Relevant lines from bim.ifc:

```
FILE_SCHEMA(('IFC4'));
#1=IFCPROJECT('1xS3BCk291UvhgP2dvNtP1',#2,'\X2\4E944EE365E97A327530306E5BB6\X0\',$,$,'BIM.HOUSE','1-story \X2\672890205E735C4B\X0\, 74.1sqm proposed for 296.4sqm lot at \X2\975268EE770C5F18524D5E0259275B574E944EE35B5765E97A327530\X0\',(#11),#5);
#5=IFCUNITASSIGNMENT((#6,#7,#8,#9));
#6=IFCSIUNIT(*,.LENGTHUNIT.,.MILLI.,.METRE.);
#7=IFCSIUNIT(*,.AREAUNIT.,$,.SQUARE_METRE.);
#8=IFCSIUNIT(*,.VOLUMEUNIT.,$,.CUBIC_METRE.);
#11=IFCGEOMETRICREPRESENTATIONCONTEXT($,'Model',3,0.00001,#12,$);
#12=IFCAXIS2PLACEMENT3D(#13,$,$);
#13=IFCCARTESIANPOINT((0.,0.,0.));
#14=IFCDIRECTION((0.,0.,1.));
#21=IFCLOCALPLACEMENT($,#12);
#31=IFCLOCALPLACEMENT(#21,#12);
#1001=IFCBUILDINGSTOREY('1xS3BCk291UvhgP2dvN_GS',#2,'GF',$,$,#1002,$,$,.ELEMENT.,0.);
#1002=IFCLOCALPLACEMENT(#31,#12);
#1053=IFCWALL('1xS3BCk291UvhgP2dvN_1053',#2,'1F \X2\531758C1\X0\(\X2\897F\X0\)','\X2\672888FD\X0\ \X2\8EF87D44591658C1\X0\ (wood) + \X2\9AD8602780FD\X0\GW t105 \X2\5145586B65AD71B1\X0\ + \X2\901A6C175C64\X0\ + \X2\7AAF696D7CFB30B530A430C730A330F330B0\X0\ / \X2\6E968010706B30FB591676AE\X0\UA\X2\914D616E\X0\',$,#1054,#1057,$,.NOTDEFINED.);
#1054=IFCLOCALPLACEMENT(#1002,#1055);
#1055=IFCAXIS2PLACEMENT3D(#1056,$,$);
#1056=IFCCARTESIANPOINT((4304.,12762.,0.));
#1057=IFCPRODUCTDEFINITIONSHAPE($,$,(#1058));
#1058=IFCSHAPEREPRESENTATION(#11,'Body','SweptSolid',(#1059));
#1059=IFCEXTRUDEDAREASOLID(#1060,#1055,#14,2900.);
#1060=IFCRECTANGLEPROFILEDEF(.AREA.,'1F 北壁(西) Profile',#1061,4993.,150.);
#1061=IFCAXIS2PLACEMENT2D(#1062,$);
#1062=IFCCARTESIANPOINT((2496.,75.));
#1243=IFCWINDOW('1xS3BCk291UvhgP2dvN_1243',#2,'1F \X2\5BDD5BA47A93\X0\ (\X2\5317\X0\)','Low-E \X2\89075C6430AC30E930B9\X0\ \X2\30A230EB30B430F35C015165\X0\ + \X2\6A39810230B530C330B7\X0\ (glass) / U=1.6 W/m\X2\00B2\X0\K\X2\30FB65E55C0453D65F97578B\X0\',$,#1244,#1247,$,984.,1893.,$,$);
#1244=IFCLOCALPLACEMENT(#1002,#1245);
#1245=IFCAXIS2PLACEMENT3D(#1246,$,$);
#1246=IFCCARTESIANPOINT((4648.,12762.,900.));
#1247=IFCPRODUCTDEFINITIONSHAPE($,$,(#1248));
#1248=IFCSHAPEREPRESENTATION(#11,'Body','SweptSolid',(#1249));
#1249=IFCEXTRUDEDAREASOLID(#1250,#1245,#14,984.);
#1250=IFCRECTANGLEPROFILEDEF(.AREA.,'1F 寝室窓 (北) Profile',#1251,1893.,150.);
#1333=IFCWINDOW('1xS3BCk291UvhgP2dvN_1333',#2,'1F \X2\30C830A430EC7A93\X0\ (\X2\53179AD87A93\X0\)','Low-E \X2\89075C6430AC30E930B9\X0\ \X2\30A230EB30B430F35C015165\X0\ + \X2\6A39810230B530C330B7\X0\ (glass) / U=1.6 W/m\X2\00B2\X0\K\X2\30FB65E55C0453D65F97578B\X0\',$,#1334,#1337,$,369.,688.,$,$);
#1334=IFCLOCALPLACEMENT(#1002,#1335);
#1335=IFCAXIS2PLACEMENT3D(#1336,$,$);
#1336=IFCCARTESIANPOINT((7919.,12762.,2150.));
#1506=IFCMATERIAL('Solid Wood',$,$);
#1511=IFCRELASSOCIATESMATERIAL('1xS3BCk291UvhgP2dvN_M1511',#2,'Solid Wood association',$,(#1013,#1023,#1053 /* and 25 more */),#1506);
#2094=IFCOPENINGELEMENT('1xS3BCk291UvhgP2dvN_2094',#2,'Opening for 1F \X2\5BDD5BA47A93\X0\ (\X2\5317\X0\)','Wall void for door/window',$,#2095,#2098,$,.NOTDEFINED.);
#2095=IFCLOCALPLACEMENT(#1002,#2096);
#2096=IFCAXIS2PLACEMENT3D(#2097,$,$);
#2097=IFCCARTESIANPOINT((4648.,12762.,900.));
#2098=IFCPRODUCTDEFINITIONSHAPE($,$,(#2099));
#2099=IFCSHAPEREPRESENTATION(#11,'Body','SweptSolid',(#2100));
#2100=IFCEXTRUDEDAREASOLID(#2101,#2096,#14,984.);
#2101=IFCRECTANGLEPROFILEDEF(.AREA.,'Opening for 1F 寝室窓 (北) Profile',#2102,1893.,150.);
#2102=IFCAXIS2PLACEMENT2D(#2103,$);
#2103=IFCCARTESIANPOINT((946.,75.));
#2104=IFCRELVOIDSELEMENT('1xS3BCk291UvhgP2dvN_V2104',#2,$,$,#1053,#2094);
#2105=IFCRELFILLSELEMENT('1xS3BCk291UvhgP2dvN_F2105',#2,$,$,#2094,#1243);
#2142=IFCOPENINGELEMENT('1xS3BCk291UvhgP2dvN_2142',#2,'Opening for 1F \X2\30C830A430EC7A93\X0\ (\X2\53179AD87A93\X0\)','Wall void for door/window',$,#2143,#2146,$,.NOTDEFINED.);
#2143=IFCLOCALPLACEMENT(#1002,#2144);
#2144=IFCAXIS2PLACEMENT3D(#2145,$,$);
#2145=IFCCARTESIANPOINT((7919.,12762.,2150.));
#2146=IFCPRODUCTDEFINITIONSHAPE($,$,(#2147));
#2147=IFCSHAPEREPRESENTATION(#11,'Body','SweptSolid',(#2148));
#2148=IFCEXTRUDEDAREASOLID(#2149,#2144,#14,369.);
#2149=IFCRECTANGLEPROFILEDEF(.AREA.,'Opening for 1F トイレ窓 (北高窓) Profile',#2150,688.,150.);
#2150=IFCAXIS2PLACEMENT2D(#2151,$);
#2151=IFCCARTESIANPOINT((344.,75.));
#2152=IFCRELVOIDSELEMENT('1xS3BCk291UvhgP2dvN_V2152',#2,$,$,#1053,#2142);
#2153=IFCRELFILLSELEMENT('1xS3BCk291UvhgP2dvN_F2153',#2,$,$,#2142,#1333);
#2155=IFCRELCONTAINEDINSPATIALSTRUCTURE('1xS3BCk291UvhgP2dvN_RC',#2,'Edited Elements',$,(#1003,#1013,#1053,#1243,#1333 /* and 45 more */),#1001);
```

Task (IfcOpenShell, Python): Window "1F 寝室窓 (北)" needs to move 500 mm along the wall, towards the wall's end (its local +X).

```python
import ifcopenshell
import ifcopenshell.api.geometry
import ifcopenshell.util.placement
import ifcopenshell.util.unit

model = ifcopenshell.open("bim.ifc")
unit_scale = ifcopenshell.util.unit.calculate_unit_scale(model)

window = model.by_id(1243)
opening = window.FillsVoids[0].RelatingOpeningElement
wall = opening.VoidsElements[0].RelatingBuildingElement

wall_matrix = ifcopenshell.util.placement.get_local_placement(wall.ObjectPlacement)
shift = wall_matrix[:3, 0] * 0.5 / unit_scale
before = ifcopenshell.util.placement.get_local_placement(window.ObjectPlacement)[:3, 3].copy()

# The window is not placed relative to its opening, so move both.
for product in (opening, window):
    matrix = ifcopenshell.util.placement.get_local_placement(product.ObjectPlacement)
    matrix[:3, 3] += shift
    ifcopenshell.api.geometry.edit_object_placement(model, product=product, matrix=matrix, is_si=False)

after = ifcopenshell.util.placement.get_local_placement(window.ObjectPlacement)[:3, 3]
print("window moved by", (after - before).round(3) + 0.0)

model.write("bim_updated.ifc")
```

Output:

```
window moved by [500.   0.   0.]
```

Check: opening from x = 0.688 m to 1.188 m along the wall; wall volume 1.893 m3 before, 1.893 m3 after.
